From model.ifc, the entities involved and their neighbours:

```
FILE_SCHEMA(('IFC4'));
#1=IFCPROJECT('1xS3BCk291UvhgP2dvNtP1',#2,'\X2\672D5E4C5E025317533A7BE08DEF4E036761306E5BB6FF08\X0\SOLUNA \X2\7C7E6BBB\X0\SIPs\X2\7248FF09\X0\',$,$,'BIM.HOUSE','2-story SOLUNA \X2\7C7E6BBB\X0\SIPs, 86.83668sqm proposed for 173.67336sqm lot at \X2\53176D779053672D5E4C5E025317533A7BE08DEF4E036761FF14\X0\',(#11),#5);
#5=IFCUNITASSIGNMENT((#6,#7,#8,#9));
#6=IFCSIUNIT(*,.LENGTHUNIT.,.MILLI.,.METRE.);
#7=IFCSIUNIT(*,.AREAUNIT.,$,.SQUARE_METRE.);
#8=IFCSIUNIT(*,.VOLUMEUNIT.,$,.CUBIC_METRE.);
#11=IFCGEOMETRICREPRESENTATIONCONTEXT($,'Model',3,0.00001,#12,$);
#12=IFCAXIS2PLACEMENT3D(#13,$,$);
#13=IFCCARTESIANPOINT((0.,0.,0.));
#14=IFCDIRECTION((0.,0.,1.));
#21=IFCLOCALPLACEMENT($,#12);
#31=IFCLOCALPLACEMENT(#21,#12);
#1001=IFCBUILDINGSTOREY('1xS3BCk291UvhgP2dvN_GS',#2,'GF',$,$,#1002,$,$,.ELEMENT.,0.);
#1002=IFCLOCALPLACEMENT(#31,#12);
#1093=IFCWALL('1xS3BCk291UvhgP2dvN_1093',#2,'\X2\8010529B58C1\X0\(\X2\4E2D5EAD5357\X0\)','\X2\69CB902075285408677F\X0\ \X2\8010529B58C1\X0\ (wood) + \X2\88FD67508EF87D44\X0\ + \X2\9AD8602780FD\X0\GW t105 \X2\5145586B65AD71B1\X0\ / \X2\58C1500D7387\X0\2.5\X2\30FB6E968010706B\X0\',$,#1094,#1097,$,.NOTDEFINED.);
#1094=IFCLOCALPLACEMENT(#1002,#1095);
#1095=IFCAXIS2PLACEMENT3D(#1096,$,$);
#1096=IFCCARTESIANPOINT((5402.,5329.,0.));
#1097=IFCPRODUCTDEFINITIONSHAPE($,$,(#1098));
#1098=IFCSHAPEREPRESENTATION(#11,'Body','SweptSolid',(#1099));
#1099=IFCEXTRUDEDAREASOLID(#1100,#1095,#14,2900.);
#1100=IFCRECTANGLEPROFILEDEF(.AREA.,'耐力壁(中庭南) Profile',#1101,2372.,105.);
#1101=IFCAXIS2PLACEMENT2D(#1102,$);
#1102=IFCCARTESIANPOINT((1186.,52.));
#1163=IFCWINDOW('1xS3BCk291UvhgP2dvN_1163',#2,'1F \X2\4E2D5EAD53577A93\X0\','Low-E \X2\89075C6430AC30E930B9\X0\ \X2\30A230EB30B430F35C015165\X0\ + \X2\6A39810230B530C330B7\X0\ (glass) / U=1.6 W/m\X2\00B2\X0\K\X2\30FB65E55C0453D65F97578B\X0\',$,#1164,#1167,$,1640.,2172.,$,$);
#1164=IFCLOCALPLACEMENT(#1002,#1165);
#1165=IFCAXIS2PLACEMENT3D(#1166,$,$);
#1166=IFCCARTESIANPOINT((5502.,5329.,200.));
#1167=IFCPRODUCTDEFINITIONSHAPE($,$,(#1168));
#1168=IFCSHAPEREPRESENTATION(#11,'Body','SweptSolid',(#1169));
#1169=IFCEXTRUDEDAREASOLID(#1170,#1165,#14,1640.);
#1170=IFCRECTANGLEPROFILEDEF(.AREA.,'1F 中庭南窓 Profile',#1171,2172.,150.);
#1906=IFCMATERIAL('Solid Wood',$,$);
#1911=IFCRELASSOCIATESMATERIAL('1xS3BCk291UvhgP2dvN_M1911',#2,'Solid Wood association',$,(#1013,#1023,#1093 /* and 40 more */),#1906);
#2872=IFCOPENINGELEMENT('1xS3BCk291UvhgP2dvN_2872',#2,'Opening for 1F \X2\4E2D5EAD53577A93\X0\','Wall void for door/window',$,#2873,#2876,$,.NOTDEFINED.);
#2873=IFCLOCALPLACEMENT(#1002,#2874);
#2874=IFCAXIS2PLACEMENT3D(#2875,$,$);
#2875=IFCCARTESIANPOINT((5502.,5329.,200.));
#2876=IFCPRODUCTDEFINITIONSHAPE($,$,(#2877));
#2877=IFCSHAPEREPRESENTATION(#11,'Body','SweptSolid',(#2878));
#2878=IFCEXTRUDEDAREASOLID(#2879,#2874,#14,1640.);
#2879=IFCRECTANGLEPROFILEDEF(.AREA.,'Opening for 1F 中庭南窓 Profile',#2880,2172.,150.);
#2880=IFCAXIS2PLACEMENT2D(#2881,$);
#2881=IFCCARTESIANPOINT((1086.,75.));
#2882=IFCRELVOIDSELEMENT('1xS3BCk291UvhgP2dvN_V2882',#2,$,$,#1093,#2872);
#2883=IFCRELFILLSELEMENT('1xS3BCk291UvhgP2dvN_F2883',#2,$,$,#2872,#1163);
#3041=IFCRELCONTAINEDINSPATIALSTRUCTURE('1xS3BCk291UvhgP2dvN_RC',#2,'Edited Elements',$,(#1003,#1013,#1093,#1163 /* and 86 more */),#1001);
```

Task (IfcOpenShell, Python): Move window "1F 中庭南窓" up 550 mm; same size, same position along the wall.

```python
import numpy as np
import ifcopenshell
import ifcopenshell.api.geometry
import ifcopenshell.util.placement
import ifcopenshell.util.unit

model = ifcopenshell.open("model.ifc")
unit_scale = ifcopenshell.util.unit.calculate_unit_scale(model)

window = model.by_id(1163)
opening = window.FillsVoids[0].RelatingOpeningElement
dz = 550.0

shift = np.array([0.0, 0.0, dz])
# The window is not placed relative to its opening, so move both.
for product in (opening, window):
    matrix = ifcopenshell.util.placement.get_local_placement(product.ObjectPlacement)
    matrix[:3, 3] += shift
    ifcopenshell.api.geometry.edit_object_placement(model, product=product, matrix=matrix, is_si=False)

print(f"moved by {dz * unit_scale:+.3f} m")

model.write("model_edited.ifc")
```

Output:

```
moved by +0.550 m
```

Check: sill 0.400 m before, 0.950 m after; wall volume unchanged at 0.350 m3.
